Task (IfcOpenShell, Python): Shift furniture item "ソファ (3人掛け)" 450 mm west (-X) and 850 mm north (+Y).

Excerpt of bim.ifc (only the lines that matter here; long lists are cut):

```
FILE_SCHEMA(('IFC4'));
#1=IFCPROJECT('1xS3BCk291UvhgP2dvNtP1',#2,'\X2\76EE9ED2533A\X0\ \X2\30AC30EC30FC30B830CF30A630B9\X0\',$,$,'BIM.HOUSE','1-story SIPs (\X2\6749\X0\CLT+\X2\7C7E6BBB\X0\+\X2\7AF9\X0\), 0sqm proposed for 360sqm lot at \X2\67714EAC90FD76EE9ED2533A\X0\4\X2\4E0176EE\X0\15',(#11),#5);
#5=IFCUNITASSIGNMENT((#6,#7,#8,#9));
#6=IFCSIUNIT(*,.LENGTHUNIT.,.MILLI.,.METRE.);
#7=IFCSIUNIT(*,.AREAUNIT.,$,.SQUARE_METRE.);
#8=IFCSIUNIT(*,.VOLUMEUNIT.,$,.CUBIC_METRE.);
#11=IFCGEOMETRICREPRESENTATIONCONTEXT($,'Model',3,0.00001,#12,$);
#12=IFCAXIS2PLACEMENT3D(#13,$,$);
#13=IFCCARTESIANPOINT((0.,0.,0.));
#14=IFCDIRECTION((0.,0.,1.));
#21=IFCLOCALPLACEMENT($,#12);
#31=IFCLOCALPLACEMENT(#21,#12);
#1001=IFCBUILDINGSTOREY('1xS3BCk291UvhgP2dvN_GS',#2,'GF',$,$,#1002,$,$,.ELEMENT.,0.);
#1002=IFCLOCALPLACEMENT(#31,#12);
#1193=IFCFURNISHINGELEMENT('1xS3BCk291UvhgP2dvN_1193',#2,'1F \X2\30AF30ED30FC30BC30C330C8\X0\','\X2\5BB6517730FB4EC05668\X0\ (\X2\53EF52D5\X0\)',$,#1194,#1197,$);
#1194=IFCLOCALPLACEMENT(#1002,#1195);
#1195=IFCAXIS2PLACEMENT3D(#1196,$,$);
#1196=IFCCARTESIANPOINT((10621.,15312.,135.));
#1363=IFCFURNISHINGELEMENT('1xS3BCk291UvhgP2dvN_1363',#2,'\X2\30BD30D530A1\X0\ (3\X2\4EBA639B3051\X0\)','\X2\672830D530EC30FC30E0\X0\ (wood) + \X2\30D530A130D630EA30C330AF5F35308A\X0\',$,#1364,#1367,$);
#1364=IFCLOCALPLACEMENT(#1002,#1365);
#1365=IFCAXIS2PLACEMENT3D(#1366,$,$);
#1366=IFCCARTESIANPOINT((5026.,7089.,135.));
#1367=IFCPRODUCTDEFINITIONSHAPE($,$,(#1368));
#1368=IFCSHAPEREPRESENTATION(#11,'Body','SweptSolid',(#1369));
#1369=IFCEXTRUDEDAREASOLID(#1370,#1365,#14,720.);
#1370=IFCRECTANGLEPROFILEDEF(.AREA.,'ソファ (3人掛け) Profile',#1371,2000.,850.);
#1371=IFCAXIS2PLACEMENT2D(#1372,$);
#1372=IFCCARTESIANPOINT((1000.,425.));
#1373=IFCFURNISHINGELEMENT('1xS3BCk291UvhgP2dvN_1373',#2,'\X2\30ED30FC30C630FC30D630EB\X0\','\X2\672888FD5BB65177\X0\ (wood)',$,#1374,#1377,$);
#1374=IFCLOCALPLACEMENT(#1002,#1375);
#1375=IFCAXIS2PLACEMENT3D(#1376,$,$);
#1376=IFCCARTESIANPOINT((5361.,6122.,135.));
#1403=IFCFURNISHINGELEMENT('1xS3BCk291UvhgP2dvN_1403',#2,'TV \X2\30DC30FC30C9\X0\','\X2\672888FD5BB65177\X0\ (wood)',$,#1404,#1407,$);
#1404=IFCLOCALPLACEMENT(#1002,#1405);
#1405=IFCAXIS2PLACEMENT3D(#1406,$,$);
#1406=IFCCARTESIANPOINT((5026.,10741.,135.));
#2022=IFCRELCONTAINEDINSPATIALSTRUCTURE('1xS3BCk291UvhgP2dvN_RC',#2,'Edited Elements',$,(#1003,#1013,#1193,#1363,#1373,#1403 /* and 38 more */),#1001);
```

```python
import ifcopenshell
import ifcopenshell.api.geometry
import ifcopenshell.util.placement

model = ifcopenshell.open("bim.ifc")

item = model.by_guid("1xS3BCk291UvhgP2dvN_1363")
matrix = ifcopenshell.util.placement.get_local_placement(item.ObjectPlacement)
matrix[0, 3] -= 450.0
matrix[1, 3] += 850.0
ifcopenshell.api.geometry.edit_object_placement(model, product=item, matrix=matrix, is_si=False)

print(ifcopenshell.util.placement.get_local_placement(item.ObjectPlacement).round(3) + 0.0)

model.write("bim_v2.ifc")
```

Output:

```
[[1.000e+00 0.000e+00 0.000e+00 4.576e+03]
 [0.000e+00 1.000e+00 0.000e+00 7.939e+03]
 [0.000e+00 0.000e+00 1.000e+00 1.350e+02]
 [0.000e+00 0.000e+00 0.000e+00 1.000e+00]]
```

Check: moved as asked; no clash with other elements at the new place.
